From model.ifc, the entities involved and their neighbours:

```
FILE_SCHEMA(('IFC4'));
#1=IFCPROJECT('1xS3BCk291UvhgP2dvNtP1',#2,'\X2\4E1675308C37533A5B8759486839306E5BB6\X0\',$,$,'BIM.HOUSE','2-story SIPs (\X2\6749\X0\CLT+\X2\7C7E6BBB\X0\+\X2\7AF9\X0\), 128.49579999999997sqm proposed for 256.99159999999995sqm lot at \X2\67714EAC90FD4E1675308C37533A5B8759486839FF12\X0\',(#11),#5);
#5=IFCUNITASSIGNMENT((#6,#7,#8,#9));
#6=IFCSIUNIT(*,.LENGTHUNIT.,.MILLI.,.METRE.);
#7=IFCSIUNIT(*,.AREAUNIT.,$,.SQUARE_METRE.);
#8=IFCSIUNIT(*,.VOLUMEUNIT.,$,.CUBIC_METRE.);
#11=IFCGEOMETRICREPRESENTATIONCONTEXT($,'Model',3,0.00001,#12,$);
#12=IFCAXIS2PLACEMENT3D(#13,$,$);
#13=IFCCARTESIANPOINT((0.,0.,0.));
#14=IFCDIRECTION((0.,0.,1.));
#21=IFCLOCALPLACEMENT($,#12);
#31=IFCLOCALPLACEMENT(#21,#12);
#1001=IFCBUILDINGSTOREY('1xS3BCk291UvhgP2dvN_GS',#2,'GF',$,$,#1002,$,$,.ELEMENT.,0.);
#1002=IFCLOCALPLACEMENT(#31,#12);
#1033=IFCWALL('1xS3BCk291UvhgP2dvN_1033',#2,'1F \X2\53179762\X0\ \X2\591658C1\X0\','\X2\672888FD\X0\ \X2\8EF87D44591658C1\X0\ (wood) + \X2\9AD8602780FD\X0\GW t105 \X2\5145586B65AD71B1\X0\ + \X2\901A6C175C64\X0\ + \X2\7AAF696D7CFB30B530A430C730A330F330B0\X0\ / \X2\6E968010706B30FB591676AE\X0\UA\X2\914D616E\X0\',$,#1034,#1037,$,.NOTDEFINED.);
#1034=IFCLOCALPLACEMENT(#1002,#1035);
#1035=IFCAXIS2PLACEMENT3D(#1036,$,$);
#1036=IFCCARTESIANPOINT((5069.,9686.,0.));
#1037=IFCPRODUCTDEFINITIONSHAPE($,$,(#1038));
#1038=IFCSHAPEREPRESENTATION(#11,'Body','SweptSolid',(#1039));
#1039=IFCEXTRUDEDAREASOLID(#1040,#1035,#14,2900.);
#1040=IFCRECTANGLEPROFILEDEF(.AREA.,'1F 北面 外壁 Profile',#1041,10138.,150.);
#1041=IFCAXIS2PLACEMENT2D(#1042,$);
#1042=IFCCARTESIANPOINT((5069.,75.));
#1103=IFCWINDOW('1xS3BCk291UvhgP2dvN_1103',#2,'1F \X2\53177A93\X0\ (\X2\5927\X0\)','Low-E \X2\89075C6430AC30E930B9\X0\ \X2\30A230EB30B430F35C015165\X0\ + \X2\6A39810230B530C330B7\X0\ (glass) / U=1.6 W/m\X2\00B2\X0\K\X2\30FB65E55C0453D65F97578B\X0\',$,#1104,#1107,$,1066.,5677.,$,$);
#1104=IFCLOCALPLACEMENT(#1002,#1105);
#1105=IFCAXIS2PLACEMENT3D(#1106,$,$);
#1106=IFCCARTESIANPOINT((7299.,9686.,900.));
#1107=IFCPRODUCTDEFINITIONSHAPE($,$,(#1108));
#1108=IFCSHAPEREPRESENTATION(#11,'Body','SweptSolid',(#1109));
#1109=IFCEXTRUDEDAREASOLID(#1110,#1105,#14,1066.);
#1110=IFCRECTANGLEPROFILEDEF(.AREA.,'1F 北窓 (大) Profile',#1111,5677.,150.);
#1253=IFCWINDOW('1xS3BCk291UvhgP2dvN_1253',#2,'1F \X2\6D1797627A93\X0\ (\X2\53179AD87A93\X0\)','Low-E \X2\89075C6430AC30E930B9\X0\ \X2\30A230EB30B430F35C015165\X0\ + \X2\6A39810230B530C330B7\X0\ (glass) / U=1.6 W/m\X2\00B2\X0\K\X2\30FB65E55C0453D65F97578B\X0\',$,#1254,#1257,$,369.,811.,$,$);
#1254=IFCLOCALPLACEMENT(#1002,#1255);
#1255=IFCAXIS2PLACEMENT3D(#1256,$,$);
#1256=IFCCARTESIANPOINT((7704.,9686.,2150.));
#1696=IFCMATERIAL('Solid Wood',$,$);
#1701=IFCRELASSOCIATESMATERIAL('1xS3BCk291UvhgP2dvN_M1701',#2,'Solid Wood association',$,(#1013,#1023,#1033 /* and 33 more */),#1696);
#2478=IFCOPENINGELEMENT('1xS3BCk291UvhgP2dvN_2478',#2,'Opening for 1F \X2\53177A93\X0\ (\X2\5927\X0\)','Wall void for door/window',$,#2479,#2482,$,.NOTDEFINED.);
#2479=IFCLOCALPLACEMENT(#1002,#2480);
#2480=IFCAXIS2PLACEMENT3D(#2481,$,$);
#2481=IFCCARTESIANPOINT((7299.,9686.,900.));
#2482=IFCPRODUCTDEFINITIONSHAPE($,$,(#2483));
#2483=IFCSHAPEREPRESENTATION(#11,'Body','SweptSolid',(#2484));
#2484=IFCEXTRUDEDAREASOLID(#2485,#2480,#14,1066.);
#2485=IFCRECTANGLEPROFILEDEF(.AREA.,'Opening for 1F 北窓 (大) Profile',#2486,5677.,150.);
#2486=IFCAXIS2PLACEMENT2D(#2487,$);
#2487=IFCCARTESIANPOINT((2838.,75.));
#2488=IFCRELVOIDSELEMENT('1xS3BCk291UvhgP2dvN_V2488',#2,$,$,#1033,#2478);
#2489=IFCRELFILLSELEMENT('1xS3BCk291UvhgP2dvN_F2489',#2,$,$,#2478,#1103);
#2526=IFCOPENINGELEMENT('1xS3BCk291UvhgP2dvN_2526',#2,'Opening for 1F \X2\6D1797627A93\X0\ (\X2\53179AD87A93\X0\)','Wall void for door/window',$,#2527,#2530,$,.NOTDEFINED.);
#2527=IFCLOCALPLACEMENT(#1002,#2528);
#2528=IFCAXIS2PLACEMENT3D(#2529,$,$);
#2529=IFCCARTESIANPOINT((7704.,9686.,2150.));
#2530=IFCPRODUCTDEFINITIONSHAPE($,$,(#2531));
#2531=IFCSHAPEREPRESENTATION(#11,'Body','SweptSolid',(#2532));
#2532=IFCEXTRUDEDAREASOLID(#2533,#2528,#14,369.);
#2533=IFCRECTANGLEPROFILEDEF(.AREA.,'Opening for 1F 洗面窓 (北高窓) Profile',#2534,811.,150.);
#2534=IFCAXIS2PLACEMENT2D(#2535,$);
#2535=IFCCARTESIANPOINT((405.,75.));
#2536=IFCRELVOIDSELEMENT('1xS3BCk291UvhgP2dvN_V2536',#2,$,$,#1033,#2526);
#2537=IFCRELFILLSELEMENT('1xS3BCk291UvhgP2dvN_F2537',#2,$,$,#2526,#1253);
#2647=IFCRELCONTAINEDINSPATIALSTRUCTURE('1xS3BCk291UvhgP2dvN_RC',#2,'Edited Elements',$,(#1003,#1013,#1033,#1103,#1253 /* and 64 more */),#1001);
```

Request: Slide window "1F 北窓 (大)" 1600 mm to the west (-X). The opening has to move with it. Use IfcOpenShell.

```python
import ifcopenshell
import ifcopenshell.api.geometry
import ifcopenshell.util.placement

model = ifcopenshell.open("model.ifc")

window = model.by_guid("1xS3BCk291UvhgP2dvN_1103")
opening = window.FillsVoids[0].RelatingOpeningElement
wall = opening.VoidsElements[0].RelatingBuildingElement

wall_matrix = ifcopenshell.util.placement.get_local_placement(wall.ObjectPlacement)
shift = wall_matrix[:3, 0] * -1600.0
before = ifcopenshell.util.placement.get_local_placement(window.ObjectPlacement)[:3, 3].copy()

# The window is not placed relative to its opening, so move both.
for product in (opening, window):
    matrix = ifcopenshell.util.placement.get_local_placement(product.ObjectPlacement)
    matrix[:3, 3] += shift
    ifcopenshell.api.geometry.edit_object_placement(model, product=product, matrix=matrix, is_si=False)

after = ifcopenshell.util.placement.get_local_placement(window.ObjectPlacement)[:3, 3]
print("window moved by", (after - before).round(3) + 0.0)

model.write("model_rev.ifc")
```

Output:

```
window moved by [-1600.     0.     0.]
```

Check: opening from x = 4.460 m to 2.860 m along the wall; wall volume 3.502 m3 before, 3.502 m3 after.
